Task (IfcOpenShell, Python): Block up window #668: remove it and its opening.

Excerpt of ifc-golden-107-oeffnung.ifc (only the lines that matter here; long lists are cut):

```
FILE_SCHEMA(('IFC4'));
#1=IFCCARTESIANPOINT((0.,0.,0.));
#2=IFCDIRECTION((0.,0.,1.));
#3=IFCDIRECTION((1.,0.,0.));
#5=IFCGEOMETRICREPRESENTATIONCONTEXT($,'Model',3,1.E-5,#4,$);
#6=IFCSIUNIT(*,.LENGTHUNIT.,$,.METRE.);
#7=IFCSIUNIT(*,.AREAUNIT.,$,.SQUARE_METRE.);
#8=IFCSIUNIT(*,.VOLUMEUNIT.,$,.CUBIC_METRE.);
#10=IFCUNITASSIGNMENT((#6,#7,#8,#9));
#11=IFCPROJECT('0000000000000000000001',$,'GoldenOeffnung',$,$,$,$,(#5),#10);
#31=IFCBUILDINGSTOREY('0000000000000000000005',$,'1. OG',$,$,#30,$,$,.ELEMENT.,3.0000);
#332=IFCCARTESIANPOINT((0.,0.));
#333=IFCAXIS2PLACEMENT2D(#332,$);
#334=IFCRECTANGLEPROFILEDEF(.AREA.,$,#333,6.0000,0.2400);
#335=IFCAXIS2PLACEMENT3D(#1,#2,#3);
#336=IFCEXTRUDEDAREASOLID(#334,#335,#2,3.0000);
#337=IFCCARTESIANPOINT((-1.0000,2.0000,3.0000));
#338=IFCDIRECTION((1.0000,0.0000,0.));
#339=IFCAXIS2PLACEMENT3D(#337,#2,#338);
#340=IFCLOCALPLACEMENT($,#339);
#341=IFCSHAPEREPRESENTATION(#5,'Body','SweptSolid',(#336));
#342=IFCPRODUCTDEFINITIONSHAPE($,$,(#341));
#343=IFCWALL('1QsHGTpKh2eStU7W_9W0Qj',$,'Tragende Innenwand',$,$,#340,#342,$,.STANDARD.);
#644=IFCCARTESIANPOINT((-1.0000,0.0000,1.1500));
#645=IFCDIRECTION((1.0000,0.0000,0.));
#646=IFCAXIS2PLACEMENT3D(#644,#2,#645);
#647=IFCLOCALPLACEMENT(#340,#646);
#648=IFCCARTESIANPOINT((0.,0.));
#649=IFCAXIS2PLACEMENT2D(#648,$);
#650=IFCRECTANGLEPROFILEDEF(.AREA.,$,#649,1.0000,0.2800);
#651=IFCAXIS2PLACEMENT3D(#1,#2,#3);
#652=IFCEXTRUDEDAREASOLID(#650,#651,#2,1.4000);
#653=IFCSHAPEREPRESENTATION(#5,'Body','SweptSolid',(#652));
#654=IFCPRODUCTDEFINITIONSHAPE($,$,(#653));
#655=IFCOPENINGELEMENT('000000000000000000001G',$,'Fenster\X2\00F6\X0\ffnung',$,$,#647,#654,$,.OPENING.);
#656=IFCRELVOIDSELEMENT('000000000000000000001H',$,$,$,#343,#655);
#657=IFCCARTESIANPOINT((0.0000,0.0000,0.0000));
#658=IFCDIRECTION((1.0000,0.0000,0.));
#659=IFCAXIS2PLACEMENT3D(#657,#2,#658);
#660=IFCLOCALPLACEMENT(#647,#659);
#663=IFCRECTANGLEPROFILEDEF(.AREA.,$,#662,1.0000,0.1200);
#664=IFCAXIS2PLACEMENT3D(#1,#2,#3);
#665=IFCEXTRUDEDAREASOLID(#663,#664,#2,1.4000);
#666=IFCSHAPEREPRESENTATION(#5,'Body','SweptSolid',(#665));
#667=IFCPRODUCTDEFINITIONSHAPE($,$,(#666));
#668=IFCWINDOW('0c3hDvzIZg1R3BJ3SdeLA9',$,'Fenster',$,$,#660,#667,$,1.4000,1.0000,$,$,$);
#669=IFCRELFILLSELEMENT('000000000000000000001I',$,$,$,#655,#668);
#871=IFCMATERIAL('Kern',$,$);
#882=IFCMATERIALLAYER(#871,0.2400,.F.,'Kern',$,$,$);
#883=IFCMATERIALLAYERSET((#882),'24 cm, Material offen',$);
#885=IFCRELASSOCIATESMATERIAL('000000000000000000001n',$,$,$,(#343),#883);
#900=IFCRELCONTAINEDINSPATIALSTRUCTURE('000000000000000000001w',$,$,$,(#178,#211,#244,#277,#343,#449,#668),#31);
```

```python
import ifcopenshell
import ifcopenshell.api.feature
import ifcopenshell.api.root
import ifcopenshell.geom
import ifcopenshell.util.shape

model = ifcopenshell.open("ifc-golden-107-oeffnung.ifc")
settings = ifcopenshell.geom.settings()


def volume(element):
    """Net volume in cubic metres, openings subtracted."""
    shape = ifcopenshell.geom.create_shape(settings, element)
    return ifcopenshell.util.shape.get_volume(shape.geometry)


window = model.by_id(668)
opening = window.FillsVoids[0].RelatingOpeningElement
wall = opening.VoidsElements[0].RelatingBuildingElement
before = volume(wall)

ifcopenshell.api.root.remove_product(model, product=window)
ifcopenshell.api.feature.remove_feature(model, feature=opening)

after = volume(wall)

print(f"wall volume {before:.3f} -> {after:.3f} m3")

model.write("ifc-golden-107-oeffnung-out.ifc")
```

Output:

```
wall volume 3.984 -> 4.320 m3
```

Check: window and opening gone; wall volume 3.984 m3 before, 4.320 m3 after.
